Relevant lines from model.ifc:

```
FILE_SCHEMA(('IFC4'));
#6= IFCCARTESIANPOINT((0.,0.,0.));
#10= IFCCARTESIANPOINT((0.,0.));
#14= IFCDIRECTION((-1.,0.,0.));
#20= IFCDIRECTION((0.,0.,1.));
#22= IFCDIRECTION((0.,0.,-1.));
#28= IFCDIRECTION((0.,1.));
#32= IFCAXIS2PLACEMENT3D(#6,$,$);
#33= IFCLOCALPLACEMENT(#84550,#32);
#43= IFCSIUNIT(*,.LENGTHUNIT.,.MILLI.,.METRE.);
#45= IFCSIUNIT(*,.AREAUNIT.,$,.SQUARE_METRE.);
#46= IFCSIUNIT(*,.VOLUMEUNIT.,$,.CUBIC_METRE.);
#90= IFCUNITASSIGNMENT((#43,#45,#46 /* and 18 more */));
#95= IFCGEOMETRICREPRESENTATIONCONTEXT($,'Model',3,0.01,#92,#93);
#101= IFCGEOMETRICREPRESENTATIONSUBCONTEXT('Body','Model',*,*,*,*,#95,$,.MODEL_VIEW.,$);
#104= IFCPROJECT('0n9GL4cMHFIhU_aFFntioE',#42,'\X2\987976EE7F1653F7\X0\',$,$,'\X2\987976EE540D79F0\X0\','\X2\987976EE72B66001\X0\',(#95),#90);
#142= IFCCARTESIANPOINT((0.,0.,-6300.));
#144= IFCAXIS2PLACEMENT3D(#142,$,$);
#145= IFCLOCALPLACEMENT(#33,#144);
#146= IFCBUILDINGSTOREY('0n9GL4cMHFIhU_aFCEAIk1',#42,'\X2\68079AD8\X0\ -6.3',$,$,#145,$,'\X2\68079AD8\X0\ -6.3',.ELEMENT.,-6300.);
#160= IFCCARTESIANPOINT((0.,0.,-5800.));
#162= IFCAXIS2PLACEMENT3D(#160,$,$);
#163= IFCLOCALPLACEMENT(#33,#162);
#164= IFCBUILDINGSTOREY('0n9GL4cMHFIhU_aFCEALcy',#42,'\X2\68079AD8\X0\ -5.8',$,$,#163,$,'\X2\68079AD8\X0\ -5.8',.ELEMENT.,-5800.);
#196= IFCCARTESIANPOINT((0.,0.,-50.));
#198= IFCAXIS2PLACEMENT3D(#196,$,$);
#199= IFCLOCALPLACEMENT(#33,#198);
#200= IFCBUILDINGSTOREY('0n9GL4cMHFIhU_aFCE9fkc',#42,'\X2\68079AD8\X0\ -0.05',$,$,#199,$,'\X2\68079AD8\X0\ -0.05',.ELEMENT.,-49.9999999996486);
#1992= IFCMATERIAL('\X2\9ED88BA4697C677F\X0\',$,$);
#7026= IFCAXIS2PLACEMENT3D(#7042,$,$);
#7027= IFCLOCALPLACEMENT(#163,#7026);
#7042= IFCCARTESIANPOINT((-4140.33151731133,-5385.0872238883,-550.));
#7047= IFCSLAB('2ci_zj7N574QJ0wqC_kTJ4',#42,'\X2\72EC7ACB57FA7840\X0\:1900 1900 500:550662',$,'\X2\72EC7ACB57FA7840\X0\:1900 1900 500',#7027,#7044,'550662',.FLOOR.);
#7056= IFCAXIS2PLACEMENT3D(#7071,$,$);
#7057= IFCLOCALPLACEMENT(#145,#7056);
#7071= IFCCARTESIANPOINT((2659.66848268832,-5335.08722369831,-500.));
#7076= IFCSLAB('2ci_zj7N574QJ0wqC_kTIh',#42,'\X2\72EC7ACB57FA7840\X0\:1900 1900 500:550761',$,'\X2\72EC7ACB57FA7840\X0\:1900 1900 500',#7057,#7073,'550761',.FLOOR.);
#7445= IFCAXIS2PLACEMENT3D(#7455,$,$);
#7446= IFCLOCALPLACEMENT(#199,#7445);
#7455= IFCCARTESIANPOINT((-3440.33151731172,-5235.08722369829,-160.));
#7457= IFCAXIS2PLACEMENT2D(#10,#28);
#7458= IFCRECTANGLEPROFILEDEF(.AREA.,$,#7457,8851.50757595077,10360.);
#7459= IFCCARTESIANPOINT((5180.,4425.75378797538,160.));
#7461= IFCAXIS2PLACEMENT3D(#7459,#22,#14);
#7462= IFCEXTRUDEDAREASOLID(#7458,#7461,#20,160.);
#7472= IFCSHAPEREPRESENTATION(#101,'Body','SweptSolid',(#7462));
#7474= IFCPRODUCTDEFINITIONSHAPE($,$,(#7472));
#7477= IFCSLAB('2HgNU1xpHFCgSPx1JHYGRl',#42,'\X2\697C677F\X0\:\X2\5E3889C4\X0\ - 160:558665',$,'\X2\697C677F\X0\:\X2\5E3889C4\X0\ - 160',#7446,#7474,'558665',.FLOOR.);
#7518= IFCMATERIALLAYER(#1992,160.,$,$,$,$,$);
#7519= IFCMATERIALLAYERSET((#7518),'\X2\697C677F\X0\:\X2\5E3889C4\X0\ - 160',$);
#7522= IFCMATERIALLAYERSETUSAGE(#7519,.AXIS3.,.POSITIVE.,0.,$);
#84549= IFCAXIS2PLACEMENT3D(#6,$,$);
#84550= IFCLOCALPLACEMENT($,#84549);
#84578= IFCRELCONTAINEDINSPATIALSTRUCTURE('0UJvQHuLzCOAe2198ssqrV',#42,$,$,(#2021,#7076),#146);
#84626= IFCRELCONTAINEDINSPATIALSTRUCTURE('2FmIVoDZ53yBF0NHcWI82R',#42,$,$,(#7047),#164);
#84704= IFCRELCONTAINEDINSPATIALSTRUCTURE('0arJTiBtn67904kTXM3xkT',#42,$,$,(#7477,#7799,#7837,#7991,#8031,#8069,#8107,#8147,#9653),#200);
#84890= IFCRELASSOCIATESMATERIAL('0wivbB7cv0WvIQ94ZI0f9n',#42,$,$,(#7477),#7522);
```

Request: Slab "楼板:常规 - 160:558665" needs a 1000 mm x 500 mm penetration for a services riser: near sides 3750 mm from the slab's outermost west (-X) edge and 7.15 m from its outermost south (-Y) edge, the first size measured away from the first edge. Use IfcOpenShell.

```python
import numpy as np
import ifcopenshell
import ifcopenshell.api.feature
import ifcopenshell.api.geometry
import ifcopenshell.api.root
import ifcopenshell.geom
import ifcopenshell.util.placement
import ifcopenshell.util.representation
import ifcopenshell.util.shape
import ifcopenshell.util.unit

model = ifcopenshell.open("model.ifc")
unit_scale = ifcopenshell.util.unit.calculate_unit_scale(model)
settings = ifcopenshell.geom.settings()


def volume(element):
    """Net volume in cubic metres, openings subtracted."""
    shape = ifcopenshell.geom.create_shape(settings, element)
    return ifcopenshell.util.shape.get_volume(shape.geometry)


slab = model.by_id(7477)
before = volume(slab)

# Extent in the slab's own axes, in metres. The edges named are its -X and -Y sides.
slab_shape = ifcopenshell.geom.create_shape(settings, slab)
vertices = ifcopenshell.util.shape.get_vertices(slab_shape.geometry)
x_min, y_min, bottom = vertices.min(axis=0)
top = vertices[:, 2].max()

opening = ifcopenshell.api.root.create_entity(model, ifc_class="IfcOpeningElement", name="Services riser opening", predefined_type="OPENING")
context = ifcopenshell.util.representation.get_context(model, "Model", "Body", "MODEL_VIEW")
width, depth = 1, 0.5
outline = [(0.0, 0.0), (width, 0.0), (width, depth), (0.0, depth), (0.0, 0.0)]
# Overshoot both faces by 50 mm so the cut is clean.
shape = ifcopenshell.api.geometry.add_slab_representation(
    model, context=context, depth=top - bottom + 0.1, polyline=outline
)
ifcopenshell.api.geometry.assign_representation(model, product=opening, representation=shape)

matrix = ifcopenshell.util.placement.get_local_placement(slab.ObjectPlacement)
matrix[:, 3] = matrix @ np.append(np.array([x_min + 3.75, y_min + 7.15, bottom - 0.05]) / unit_scale, 1.0)
ifcopenshell.api.geometry.edit_object_placement(model, product=opening, matrix=matrix, is_si=False)
ifcopenshell.api.feature.add_feature(model, feature=opening, element=slab)

after = volume(slab)

print(f"slab volume {before:.3f} -> {after:.3f} m3")

model.write("model_v2.ifc")
```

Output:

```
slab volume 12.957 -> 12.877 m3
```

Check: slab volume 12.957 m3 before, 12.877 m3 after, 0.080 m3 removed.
